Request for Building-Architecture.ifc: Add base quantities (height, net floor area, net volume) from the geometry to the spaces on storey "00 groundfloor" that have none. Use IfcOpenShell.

First a look at what the model holds.

```python
import ifcopenshell
import ifcopenshell.util.element
import ifcopenshell.util.unit

model = ifcopenshell.open("Building-Architecture.ifc")
print(model.schema)
for unit_type in ("LENGTHUNIT", "AREAUNIT", "VOLUMEUNIT"):
    print(unit_type, ifcopenshell.util.unit.calculate_unit_scale(model, unit_type))
storey = next(s for s in model.by_type("IfcBuildingStorey") if s.Name == "00 groundfloor")
spaces = [e for e in ifcopenshell.util.element.get_decomposition(storey) if e.is_a("IfcSpace")]
for e in sorted(spaces, key=lambda e: e.id()):
    print(e.id(), e.is_a(), e.Name, list(ifcopenshell.util.element.get_psets(e, qtos_only=True)), sep=" | ")
```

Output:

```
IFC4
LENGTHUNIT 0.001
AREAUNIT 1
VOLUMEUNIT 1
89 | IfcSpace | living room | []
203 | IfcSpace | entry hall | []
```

```python
import ifcopenshell
import ifcopenshell.api.pset
import ifcopenshell.geom
import ifcopenshell.util.element
import ifcopenshell.util.shape
import ifcopenshell.util.unit

model = ifcopenshell.open("Building-Architecture.ifc")
unit_scale = ifcopenshell.util.unit.calculate_unit_scale(model)
area_scale = ifcopenshell.util.unit.calculate_unit_scale(model, "AREAUNIT")
volume_scale = ifcopenshell.util.unit.calculate_unit_scale(model, "VOLUMEUNIT")
settings = ifcopenshell.geom.settings()

storey = next(s for s in model.by_type("IfcBuildingStorey") if s.Name == "00 groundfloor")
spaces = [e for e in ifcopenshell.util.element.get_decomposition(storey) if e.is_a("IfcSpace")]

for e in sorted(spaces, key=lambda e: e.id()):
    if ifcopenshell.util.element.get_psets(e, qtos_only=True, should_inherit=False):
        continue
    # Geometry comes back in metres, in the element's own axes.
    shape = ifcopenshell.geom.create_shape(settings, e)
    values = {
        "Height": ifcopenshell.util.shape.get_z(shape.geometry) / unit_scale,
        "NetFloorArea": ifcopenshell.util.shape.get_footprint_area(shape.geometry) / area_scale,
        "NetVolume": ifcopenshell.util.shape.get_volume(shape.geometry) / volume_scale,
    }
    qto = ifcopenshell.api.pset.add_qto(model, product=e, name="Qto_SpaceBaseQuantities")
    ifcopenshell.api.pset.edit_qto(model, qto=qto, properties=values)
    print(e.id(), {k: round(v, 3) for k, v in values.items()})

model.write("Building-Architecture_v2.ifc")
```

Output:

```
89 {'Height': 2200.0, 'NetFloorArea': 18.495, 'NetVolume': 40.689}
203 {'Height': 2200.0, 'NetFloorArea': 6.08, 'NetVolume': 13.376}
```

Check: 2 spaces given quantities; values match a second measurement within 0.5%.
